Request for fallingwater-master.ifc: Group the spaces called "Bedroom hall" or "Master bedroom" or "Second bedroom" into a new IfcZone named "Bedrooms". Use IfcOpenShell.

First a look at what the model holds.

```python
import ifcopenshell

model = ifcopenshell.open("fallingwater-master.ifc")
print(model.schema)
seen = {}
for space in model.by_type("IfcSpace"):
    seen[space.LongName] = seen.get(space.LongName, 0) + 1
for name, count in sorted(seen.items(), key=str):
    print(count, "x", name)
print("zones:", [z.Name for z in model.by_type("IfcZone")][:20])
```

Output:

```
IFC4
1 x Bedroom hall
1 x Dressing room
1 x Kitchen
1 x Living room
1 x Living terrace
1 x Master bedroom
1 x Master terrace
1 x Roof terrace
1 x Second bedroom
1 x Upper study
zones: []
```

```python
import ifcopenshell
import ifcopenshell.api.group
import ifcopenshell.api.root

model = ifcopenshell.open("fallingwater-master.ifc")

names = {"Bedroom hall", "Master bedroom", "Second bedroom"}
spaces = [s for s in model.by_type("IfcSpace") if s.LongName in names]

zone = ifcopenshell.api.root.create_entity(model, ifc_class="IfcZone", name="Bedrooms")
ifcopenshell.api.group.assign_group(model, products=spaces, group=zone)
print(len(spaces), "spaces in", zone.Name)

model.write("fallingwater-master_rev.ifc")
```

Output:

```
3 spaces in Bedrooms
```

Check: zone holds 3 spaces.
